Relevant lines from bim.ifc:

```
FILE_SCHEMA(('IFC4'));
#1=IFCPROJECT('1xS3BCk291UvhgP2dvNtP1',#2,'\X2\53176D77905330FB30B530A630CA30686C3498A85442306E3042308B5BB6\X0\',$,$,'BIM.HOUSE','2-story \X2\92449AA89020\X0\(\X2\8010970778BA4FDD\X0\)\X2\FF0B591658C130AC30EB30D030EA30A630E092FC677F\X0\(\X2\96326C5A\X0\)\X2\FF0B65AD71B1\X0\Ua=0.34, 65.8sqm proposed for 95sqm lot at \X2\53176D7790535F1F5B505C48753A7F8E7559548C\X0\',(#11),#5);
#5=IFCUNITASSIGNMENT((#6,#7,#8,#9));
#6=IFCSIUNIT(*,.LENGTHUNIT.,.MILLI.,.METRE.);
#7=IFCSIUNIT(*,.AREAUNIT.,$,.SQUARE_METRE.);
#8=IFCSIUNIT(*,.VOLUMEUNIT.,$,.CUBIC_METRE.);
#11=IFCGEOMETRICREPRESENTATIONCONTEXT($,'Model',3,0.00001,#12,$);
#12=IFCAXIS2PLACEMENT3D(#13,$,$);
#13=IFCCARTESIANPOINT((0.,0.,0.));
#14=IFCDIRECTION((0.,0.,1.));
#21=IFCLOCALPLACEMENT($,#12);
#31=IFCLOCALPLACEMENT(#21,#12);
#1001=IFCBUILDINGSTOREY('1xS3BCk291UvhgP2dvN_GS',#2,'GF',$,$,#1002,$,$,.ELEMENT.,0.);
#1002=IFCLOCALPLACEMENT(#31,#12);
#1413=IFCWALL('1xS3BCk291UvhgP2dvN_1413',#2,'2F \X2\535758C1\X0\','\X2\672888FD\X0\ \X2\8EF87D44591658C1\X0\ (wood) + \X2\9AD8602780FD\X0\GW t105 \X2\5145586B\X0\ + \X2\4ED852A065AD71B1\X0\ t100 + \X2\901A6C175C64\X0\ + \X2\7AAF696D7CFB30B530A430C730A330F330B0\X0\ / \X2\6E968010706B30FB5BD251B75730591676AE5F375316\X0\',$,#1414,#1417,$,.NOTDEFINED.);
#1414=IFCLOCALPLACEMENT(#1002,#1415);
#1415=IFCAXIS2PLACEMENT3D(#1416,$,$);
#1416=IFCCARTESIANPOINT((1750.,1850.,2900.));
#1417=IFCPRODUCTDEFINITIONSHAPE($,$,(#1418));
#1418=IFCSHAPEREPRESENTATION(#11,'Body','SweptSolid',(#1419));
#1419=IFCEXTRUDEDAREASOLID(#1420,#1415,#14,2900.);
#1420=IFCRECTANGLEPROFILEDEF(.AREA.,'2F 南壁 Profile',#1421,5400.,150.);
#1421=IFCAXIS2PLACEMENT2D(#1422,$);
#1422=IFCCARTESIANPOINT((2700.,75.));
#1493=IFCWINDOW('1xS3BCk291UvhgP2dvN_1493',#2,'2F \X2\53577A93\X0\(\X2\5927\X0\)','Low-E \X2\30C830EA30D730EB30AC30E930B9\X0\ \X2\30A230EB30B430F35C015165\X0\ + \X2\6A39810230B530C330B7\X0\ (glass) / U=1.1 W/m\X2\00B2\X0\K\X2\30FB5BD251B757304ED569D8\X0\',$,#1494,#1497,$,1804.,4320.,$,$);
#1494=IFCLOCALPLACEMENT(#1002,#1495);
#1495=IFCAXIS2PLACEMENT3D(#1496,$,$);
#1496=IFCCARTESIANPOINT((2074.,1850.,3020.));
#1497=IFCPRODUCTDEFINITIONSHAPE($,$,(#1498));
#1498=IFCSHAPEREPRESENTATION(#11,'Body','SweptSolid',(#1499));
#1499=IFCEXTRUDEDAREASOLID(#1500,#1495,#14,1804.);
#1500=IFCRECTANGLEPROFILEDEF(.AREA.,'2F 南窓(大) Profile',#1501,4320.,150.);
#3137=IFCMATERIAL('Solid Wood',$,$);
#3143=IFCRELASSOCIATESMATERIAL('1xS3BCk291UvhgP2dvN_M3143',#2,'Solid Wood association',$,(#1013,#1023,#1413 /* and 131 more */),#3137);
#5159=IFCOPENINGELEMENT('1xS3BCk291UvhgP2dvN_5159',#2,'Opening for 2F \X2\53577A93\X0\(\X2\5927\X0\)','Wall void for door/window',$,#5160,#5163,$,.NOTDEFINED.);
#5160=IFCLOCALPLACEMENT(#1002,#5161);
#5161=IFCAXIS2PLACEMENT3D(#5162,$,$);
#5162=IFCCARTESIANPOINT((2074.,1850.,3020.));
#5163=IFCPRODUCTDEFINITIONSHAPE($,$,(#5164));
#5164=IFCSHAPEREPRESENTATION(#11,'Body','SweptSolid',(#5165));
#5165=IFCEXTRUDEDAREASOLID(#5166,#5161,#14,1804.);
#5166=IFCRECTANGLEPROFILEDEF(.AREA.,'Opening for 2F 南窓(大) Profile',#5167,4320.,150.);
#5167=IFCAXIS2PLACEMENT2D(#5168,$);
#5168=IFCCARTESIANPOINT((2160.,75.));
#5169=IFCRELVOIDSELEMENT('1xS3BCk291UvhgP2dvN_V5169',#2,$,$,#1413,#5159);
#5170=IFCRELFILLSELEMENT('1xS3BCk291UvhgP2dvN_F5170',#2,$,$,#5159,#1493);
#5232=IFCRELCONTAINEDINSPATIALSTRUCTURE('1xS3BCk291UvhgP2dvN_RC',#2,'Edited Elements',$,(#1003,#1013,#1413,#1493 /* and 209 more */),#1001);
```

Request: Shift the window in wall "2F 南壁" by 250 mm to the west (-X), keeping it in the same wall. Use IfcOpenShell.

```python
import ifcopenshell
import ifcopenshell.api.geometry
import ifcopenshell.util.placement
import ifcopenshell.util.unit

model = ifcopenshell.open("bim.ifc")
unit_scale = ifcopenshell.util.unit.calculate_unit_scale(model)

window = model.by_id(1493)
opening = window.FillsVoids[0].RelatingOpeningElement
wall = opening.VoidsElements[0].RelatingBuildingElement

wall_matrix = ifcopenshell.util.placement.get_local_placement(wall.ObjectPlacement)
shift = wall_matrix[:3, 0] * -0.25 / unit_scale
before = ifcopenshell.util.placement.get_local_placement(window.ObjectPlacement)[:3, 3].copy()

# The window is not placed relative to its opening, so move both.
for product in (opening, window):
    matrix = ifcopenshell.util.placement.get_local_placement(product.ObjectPlacement)
    matrix[:3, 3] += shift
    ifcopenshell.api.geometry.edit_object_placement(model, product=product, matrix=matrix, is_si=False)

after = ifcopenshell.util.placement.get_local_placement(window.ObjectPlacement)[:3, 3]
print("window moved by", (after - before).round(3) + 0.0)

model.write("bim_updated.ifc")
```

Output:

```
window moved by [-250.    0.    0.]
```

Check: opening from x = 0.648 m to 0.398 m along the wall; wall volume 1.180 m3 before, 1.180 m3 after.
